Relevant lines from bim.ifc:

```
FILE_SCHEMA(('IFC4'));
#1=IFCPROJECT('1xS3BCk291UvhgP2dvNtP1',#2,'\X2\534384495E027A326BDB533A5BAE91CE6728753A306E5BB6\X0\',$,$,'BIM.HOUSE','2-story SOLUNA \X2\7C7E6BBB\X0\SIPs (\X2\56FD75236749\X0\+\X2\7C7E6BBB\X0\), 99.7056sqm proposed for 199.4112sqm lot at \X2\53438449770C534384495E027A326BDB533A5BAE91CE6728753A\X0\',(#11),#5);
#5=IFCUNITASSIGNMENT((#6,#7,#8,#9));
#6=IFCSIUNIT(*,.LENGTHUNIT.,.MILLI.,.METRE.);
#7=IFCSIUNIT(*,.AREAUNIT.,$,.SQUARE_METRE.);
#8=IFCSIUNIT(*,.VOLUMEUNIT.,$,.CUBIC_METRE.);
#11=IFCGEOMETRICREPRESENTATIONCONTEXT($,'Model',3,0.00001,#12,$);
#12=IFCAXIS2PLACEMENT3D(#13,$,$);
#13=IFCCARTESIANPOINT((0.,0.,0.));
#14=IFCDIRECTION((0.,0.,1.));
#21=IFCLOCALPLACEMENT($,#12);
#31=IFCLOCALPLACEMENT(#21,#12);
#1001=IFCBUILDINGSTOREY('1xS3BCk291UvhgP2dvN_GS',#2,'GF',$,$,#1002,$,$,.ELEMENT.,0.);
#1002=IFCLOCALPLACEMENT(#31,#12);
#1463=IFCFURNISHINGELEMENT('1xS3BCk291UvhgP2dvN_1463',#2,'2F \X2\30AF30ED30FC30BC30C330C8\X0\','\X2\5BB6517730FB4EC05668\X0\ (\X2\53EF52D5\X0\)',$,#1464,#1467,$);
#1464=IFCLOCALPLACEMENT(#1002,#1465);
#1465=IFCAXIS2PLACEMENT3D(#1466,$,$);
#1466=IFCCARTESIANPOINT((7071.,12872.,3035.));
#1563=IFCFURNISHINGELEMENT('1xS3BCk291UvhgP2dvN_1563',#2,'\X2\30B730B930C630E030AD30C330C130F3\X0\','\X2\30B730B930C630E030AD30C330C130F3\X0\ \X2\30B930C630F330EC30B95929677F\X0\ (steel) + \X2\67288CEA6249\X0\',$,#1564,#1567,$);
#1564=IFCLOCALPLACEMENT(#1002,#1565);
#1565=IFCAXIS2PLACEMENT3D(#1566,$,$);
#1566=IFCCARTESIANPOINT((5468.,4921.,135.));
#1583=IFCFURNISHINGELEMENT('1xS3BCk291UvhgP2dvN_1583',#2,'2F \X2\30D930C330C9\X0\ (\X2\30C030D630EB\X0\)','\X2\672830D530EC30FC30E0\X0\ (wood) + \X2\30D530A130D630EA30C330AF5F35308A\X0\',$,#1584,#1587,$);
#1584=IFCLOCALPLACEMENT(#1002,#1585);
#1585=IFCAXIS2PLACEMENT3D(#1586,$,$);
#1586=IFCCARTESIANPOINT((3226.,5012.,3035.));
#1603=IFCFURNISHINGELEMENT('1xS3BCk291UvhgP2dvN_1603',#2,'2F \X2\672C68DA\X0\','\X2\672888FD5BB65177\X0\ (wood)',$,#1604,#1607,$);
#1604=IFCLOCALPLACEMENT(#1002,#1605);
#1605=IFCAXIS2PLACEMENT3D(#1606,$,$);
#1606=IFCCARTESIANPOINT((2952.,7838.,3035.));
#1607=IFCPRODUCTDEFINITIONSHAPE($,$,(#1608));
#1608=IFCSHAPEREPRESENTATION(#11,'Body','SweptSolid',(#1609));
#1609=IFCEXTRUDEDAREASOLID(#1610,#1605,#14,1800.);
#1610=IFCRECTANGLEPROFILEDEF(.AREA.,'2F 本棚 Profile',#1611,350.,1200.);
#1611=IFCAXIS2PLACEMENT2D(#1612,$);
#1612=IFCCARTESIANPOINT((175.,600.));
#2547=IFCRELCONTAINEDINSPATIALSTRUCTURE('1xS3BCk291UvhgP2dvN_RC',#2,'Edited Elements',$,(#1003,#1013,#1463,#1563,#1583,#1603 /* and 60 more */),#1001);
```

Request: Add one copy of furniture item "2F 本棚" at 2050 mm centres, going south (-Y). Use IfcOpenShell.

```python
import numpy as np
import ifcopenshell
import ifcopenshell.api.geometry
import ifcopenshell.api.root
import ifcopenshell.util.element
import ifcopenshell.util.placement
import ifcopenshell.util.unit

model = ifcopenshell.open("bim.ifc")
unit_scale = ifcopenshell.util.unit.calculate_unit_scale(model)


def reuse_history(source, copy):
    """copy_class also copies each property set's owner history, people and application; keep the originals."""
    for rel in copy.IsDefinedBy:
        if rel.is_a("IfcRelDefinesByProperties") and (history := rel.RelatingPropertyDefinition.OwnerHistory):
            rel.RelatingPropertyDefinition.OwnerHistory = source.OwnerHistory
            ifcopenshell.util.element.remove_deep2(model, history)


source = model.by_guid("1xS3BCk291UvhgP2dvN_1603")
base = ifcopenshell.util.placement.get_local_placement(source.ObjectPlacement)
step = np.array([0.0, -1.0, 0.0]) * 2.05 / unit_scale

for i in range(1, 2):
    copy = ifcopenshell.api.root.copy_class(model, product=source)
    copy.Representation = ifcopenshell.util.element.copy_deep(
        model, source.Representation, exclude=["IfcGeometricRepresentationContext", "IfcRepresentationMap"]
    )
    reuse_history(source, copy)
    matrix = base.copy()
    matrix[:3, 3] += i * step
    print("added at", matrix[:3, 3].round(3) + 0.0)
    ifcopenshell.api.geometry.edit_object_placement(model, product=copy, matrix=matrix, is_si=False)

model.write("bim_rev.ifc")
```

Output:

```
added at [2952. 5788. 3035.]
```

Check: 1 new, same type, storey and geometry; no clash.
